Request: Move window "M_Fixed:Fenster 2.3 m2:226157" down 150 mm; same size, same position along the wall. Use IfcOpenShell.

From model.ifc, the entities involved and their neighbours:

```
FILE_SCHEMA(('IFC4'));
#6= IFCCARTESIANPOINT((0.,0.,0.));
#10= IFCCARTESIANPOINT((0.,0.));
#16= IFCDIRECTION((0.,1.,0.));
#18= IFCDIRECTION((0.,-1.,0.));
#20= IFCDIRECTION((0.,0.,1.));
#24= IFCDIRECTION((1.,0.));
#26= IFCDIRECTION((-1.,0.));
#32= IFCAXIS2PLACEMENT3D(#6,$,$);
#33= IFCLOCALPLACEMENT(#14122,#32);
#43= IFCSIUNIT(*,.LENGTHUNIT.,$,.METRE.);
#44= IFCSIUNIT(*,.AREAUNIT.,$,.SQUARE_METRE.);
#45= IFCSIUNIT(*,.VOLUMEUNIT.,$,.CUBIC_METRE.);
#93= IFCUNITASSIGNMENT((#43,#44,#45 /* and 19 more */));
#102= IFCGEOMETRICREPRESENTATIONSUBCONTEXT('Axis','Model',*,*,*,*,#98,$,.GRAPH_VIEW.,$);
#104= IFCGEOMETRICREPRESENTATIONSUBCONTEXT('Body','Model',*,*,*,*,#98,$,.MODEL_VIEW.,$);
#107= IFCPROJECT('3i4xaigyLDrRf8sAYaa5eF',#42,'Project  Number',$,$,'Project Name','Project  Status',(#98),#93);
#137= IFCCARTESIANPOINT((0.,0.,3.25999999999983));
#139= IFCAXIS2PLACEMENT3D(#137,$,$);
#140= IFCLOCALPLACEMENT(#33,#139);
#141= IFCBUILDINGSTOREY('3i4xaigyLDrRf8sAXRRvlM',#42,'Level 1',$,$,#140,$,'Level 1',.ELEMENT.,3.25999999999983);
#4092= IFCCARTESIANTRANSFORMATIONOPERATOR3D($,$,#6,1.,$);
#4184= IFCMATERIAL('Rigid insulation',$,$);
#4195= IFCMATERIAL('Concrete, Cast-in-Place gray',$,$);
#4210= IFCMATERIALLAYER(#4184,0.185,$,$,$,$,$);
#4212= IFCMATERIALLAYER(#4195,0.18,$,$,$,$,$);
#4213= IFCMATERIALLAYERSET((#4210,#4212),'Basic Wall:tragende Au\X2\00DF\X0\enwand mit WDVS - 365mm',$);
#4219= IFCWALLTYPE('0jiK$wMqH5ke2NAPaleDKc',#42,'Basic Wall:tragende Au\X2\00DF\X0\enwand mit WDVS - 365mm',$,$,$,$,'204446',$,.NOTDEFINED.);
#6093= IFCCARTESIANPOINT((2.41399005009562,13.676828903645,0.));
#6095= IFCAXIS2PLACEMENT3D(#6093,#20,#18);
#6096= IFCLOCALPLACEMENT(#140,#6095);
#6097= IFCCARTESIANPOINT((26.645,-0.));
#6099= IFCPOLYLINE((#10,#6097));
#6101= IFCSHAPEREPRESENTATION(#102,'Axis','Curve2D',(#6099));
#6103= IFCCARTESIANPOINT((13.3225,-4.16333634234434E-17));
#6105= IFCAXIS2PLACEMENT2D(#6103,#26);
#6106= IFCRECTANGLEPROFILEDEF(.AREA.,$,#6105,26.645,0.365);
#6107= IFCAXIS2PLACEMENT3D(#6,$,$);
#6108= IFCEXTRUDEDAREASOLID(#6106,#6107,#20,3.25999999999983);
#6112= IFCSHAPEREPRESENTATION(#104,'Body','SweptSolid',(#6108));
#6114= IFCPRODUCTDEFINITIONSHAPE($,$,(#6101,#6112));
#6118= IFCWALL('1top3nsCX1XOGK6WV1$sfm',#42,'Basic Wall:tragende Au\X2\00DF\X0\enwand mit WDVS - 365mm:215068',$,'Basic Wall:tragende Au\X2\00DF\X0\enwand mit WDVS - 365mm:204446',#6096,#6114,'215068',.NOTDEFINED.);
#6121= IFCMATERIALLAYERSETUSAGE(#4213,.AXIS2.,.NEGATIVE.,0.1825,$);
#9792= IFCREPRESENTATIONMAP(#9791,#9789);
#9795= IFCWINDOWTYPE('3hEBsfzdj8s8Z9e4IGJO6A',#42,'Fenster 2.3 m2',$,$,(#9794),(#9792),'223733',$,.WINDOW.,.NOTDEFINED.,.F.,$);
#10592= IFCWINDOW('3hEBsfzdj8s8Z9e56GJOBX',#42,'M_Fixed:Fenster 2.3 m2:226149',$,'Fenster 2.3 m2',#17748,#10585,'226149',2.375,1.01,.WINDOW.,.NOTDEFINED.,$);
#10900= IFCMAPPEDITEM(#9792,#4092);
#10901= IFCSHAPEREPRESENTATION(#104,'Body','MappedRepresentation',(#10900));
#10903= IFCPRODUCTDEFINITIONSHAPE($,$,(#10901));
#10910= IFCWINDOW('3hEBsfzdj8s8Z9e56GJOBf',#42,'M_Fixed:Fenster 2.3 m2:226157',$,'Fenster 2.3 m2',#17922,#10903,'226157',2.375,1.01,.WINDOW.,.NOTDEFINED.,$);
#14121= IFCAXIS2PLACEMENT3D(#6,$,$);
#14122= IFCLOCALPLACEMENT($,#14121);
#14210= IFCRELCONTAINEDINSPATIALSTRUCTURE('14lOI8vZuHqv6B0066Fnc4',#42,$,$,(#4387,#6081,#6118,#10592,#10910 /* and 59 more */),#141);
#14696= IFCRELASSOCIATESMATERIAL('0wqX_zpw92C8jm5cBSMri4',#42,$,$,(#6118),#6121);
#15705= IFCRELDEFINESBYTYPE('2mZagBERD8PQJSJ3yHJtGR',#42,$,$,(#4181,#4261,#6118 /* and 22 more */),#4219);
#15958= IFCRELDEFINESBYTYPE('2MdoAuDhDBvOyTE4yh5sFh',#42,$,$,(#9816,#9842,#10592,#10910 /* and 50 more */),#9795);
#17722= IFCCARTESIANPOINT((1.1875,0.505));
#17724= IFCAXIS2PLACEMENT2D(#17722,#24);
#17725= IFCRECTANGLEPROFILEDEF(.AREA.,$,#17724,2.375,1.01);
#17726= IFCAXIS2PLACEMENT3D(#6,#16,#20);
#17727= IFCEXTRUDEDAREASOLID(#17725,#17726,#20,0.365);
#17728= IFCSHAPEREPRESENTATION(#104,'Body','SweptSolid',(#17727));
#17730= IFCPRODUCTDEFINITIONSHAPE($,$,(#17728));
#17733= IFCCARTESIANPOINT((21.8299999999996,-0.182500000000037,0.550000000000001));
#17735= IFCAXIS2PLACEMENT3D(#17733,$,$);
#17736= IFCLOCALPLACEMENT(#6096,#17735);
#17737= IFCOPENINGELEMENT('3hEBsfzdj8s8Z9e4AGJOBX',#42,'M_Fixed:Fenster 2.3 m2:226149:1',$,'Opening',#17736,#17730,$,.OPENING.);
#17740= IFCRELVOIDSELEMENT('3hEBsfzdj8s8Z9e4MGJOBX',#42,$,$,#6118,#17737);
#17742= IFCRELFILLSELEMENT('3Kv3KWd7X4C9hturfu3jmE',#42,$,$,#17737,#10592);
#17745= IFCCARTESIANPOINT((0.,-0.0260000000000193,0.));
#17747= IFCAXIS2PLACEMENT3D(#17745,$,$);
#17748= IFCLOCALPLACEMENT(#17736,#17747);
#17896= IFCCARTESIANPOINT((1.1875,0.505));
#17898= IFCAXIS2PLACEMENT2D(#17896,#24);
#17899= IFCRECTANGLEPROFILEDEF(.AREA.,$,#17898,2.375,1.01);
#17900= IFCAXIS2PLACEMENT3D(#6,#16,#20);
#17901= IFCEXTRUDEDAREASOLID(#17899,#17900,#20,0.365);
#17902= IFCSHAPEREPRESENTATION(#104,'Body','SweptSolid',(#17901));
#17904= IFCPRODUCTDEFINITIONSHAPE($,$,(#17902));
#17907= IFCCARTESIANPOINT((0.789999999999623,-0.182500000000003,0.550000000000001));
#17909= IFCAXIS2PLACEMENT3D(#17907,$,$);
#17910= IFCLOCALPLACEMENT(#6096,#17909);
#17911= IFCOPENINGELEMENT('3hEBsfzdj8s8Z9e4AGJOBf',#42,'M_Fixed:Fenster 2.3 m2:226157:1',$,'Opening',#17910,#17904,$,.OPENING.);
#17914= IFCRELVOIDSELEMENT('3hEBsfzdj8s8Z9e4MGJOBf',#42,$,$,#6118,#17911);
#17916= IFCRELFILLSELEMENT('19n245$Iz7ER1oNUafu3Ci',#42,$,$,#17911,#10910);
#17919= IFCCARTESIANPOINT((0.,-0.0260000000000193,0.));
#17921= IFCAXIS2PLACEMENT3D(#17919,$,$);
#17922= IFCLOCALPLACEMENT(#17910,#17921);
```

```python
import numpy as np
import ifcopenshell
import ifcopenshell.api.geometry
import ifcopenshell.util.placement
import ifcopenshell.util.unit

model = ifcopenshell.open("model.ifc")
unit_scale = ifcopenshell.util.unit.calculate_unit_scale(model)

window = model.by_id(10910)
opening = window.FillsVoids[0].RelatingOpeningElement
dz = -0.15

shift = np.array([0.0, 0.0, dz])
# The window is placed relative to its opening, so it follows when the opening moves.
matrix = ifcopenshell.util.placement.get_local_placement(opening.ObjectPlacement)
matrix[:3, 3] += shift
ifcopenshell.api.geometry.edit_object_placement(
    model, product=opening, matrix=matrix, is_si=False, should_transform_children=True
)

print(f"moved by {dz * unit_scale:+.3f} m")

model.write("model-out.ifc")
```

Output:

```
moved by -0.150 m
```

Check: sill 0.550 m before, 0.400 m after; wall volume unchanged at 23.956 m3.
